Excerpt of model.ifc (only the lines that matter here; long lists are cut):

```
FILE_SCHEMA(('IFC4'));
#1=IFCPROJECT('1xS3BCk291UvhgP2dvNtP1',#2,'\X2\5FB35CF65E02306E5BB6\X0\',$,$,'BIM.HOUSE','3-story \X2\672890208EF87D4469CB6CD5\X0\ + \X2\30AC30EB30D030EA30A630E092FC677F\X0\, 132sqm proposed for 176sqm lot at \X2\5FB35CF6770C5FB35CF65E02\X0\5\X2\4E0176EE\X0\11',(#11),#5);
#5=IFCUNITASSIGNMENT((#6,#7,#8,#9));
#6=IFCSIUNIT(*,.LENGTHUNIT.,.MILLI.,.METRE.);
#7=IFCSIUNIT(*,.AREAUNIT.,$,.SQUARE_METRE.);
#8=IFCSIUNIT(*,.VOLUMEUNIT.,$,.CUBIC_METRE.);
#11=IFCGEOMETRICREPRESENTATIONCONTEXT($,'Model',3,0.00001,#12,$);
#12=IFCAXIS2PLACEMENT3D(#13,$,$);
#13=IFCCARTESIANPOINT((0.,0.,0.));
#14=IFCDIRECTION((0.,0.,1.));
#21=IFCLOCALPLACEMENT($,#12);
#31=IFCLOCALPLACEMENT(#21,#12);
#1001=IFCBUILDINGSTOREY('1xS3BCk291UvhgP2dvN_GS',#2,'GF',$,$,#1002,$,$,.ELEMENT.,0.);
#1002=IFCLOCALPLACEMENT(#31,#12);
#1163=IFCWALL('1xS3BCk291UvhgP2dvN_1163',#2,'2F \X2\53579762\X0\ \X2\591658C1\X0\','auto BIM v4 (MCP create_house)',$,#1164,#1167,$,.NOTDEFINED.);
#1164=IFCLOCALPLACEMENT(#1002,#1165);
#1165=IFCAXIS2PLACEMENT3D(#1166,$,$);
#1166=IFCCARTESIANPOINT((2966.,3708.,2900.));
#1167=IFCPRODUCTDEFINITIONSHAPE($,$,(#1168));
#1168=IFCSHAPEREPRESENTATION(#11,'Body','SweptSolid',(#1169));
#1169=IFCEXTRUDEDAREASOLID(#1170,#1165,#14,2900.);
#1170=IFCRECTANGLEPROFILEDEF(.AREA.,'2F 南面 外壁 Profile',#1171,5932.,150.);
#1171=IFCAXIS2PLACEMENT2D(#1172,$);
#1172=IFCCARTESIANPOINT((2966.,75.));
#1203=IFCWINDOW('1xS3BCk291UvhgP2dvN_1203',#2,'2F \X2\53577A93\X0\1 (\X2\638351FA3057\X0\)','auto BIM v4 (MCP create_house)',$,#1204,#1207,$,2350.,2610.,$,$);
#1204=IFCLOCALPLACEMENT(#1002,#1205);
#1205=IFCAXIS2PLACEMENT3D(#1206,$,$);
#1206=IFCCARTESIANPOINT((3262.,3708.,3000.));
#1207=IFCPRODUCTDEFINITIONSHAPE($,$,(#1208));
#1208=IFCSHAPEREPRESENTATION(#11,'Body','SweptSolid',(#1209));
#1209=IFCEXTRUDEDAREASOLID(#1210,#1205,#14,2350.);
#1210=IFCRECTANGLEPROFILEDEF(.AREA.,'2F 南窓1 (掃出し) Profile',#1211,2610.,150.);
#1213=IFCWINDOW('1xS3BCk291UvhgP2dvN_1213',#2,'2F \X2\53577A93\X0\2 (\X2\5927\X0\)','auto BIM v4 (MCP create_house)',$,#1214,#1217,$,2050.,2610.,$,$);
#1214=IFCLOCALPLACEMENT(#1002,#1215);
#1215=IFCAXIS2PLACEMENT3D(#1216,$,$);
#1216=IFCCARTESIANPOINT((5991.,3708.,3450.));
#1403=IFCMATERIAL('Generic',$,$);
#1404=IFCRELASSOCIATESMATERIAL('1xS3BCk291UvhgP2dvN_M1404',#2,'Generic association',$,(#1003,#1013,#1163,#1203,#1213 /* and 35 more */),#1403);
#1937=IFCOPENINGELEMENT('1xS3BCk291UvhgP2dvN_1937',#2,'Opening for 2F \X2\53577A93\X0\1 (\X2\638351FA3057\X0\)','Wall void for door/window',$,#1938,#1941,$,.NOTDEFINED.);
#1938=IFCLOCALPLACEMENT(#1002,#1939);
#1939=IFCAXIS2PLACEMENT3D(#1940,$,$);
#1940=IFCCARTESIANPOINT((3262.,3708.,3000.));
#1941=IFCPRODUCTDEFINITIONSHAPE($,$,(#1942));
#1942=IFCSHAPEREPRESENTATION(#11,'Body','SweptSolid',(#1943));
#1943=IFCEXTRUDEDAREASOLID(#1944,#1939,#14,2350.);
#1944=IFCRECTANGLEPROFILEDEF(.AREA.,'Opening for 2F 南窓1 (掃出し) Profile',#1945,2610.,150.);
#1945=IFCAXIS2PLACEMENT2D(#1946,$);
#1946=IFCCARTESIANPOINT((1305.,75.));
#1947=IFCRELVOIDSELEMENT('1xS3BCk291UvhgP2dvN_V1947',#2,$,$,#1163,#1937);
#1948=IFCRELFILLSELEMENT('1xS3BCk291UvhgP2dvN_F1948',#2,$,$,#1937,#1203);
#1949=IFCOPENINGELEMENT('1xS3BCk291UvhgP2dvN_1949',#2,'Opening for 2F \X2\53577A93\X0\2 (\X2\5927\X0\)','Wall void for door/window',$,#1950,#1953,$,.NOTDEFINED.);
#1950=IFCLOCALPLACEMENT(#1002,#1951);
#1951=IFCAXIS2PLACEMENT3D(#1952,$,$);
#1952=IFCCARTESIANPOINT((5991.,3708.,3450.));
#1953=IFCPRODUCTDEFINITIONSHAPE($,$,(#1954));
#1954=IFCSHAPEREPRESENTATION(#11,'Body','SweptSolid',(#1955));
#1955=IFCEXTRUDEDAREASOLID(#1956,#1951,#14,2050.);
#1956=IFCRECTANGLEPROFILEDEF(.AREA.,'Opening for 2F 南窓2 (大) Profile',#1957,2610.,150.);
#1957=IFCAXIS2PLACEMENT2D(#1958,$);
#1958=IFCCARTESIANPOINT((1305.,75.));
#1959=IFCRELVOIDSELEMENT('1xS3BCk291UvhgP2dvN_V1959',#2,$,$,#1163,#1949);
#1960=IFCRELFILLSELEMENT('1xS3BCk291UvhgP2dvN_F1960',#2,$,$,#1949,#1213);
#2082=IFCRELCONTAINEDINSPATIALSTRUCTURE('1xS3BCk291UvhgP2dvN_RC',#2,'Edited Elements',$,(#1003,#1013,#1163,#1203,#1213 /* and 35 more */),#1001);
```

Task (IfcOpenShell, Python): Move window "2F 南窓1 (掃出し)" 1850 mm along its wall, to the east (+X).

```python
import ifcopenshell
import ifcopenshell.api.geometry
import ifcopenshell.util.placement
import ifcopenshell.util.unit

model = ifcopenshell.open("model.ifc")
unit_scale = ifcopenshell.util.unit.calculate_unit_scale(model)

window = model.by_guid("1xS3BCk291UvhgP2dvN_1203")
opening = window.FillsVoids[0].RelatingOpeningElement
wall = opening.VoidsElements[0].RelatingBuildingElement

wall_matrix = ifcopenshell.util.placement.get_local_placement(wall.ObjectPlacement)
shift = wall_matrix[:3, 0] * 1.85 / unit_scale
before = ifcopenshell.util.placement.get_local_placement(window.ObjectPlacement)[:3, 3].copy()

# The window is not placed relative to its opening, so move both.
for product in (opening, window):
    matrix = ifcopenshell.util.placement.get_local_placement(product.ObjectPlacement)
    matrix[:3, 3] += shift
    ifcopenshell.api.geometry.edit_object_placement(model, product=product, matrix=matrix, is_si=False)

after = ifcopenshell.util.placement.get_local_placement(window.ObjectPlacement)[:3, 3]
print("window moved by", (after - before).round(3) + 0.0)

model.write("model-out.ifc")
```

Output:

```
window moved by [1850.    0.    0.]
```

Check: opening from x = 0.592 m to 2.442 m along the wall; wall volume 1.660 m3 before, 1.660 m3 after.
